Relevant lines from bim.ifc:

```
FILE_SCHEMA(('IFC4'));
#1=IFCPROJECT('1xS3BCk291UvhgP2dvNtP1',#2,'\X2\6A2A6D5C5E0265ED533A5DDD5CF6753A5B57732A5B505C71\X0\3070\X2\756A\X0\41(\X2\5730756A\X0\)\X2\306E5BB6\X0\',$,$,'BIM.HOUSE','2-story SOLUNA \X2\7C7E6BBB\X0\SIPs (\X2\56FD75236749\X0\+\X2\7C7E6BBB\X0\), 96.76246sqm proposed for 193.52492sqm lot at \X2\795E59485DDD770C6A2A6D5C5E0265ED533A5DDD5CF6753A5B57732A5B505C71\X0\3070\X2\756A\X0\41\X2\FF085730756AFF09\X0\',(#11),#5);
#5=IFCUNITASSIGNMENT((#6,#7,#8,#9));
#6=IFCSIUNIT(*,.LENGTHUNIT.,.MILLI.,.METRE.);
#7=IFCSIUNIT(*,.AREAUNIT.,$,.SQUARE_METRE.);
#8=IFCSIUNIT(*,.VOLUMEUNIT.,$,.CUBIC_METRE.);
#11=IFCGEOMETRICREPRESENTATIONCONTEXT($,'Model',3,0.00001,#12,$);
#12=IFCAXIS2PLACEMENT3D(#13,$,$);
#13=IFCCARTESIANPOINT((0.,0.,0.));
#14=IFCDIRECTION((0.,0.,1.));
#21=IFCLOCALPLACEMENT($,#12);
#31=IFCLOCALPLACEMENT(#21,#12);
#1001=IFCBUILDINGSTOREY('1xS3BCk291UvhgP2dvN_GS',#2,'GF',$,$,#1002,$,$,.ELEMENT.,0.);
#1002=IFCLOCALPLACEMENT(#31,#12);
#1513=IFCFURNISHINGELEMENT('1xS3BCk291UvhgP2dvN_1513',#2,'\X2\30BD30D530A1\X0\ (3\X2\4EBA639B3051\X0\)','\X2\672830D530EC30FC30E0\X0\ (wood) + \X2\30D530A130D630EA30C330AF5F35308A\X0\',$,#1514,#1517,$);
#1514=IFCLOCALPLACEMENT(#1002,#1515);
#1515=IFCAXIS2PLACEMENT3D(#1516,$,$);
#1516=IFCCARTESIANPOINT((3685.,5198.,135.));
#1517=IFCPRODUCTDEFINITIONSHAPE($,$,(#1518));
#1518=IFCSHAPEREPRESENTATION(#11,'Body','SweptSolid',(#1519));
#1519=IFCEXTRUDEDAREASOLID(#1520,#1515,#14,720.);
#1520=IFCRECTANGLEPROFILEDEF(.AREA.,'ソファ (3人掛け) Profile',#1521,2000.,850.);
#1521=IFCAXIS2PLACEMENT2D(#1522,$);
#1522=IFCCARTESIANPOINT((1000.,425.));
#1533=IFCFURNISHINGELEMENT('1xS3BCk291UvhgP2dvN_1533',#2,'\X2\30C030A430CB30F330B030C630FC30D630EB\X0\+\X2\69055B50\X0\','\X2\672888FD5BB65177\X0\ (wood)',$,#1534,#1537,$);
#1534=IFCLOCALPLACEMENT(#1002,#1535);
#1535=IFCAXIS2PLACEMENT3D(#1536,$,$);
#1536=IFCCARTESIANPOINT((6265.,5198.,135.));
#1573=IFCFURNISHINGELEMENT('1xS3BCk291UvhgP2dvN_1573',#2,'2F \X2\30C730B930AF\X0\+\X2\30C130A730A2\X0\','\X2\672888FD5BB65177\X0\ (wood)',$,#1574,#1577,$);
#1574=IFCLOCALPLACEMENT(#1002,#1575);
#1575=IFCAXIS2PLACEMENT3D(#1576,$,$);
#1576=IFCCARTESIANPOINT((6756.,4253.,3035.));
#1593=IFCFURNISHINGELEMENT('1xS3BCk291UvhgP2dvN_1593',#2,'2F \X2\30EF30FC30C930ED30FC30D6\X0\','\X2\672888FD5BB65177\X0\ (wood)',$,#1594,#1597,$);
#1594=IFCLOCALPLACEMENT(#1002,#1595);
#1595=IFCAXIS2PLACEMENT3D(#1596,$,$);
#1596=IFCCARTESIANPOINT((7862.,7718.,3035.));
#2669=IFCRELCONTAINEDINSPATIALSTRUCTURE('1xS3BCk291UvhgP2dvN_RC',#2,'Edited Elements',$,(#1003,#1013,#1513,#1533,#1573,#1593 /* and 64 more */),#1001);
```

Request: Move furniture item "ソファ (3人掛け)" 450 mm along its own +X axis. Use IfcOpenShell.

```python
import ifcopenshell
import ifcopenshell.api.geometry
import ifcopenshell.util.placement
import ifcopenshell.util.unit

model = ifcopenshell.open("bim.ifc")
unit_scale = ifcopenshell.util.unit.calculate_unit_scale(model)

item = model.by_guid("1xS3BCk291UvhgP2dvN_1513")
matrix = ifcopenshell.util.placement.get_local_placement(item.ObjectPlacement)
matrix[:3, 3] += matrix[:3, 0] * 0.45 / unit_scale
ifcopenshell.api.geometry.edit_object_placement(model, product=item, matrix=matrix, is_si=False)

print(ifcopenshell.util.placement.get_local_placement(item.ObjectPlacement).round(3) + 0.0)

model.write("bim_edited.ifc")
```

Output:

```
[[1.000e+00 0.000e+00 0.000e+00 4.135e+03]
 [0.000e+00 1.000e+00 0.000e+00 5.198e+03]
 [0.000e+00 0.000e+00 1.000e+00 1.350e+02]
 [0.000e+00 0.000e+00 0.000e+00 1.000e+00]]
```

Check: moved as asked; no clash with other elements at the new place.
